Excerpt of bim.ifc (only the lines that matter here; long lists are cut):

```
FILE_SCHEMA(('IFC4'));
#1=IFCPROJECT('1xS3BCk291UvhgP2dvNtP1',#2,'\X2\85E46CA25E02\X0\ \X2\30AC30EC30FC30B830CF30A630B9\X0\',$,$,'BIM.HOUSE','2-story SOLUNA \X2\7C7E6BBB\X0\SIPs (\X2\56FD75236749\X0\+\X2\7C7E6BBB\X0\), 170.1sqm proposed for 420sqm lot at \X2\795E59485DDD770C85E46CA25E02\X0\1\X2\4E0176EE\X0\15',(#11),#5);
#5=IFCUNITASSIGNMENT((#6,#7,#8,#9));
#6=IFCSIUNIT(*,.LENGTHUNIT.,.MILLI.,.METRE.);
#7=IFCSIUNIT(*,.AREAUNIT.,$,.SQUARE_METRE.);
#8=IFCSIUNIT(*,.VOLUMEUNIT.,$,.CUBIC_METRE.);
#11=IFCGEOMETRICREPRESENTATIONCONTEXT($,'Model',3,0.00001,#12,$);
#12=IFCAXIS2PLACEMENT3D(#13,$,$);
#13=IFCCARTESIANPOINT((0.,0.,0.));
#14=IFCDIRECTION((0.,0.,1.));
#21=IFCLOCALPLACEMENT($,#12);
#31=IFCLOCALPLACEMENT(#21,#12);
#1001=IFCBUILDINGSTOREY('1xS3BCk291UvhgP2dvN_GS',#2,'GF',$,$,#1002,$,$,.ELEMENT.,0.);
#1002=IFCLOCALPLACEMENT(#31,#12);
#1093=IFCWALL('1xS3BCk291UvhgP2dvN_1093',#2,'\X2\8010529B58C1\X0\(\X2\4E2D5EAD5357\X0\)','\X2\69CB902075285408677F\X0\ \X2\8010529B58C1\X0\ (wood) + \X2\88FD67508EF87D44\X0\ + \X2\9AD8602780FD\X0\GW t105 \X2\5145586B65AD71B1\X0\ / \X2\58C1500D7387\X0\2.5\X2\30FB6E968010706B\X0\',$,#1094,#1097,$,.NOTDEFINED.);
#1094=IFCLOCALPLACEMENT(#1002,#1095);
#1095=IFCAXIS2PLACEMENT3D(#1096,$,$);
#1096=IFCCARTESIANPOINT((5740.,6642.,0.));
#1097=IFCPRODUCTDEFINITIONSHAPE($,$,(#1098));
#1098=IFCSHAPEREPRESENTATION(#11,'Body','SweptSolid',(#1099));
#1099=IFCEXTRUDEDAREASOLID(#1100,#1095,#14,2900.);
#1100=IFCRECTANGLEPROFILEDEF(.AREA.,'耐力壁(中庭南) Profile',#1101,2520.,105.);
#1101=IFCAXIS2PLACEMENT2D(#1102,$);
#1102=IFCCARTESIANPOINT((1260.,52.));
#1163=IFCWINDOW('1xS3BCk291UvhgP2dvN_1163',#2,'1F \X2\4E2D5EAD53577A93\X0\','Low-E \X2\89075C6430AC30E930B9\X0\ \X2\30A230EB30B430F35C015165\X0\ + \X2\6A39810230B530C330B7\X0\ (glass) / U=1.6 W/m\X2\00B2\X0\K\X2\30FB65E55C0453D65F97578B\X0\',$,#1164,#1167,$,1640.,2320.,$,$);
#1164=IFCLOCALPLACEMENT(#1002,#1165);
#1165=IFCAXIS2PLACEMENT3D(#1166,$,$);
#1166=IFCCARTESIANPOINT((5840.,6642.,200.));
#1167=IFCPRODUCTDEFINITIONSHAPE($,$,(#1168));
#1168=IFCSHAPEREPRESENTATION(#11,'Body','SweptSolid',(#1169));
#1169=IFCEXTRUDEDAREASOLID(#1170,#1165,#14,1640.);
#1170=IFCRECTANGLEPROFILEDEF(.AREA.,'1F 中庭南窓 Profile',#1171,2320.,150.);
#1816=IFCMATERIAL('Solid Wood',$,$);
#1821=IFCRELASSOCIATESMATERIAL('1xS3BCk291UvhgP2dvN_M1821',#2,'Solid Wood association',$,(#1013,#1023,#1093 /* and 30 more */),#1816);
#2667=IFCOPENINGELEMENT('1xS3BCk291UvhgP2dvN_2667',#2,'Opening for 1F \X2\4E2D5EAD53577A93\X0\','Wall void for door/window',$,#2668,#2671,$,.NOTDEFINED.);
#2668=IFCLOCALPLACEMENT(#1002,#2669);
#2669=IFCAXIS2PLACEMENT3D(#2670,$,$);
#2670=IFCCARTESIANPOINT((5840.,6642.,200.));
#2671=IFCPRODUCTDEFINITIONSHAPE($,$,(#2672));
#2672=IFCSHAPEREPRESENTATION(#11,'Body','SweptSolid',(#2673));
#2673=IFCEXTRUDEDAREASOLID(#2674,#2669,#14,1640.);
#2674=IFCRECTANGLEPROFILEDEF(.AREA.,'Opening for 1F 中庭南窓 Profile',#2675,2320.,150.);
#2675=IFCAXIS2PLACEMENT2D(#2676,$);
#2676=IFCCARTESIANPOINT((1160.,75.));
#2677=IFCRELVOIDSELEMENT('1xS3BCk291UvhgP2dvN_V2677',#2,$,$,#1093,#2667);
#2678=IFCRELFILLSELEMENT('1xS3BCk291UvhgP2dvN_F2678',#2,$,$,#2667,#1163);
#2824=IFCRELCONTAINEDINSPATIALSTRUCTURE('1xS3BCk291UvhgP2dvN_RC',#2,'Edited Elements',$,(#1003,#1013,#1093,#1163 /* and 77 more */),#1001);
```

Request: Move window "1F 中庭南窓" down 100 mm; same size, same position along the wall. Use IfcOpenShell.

```python
import numpy as np
import ifcopenshell
import ifcopenshell.api.geometry
import ifcopenshell.util.placement
import ifcopenshell.util.unit

model = ifcopenshell.open("bim.ifc")
unit_scale = ifcopenshell.util.unit.calculate_unit_scale(model)

window = model.by_guid("1xS3BCk291UvhgP2dvN_1163")
opening = window.FillsVoids[0].RelatingOpeningElement
dz = -100.0

shift = np.array([0.0, 0.0, dz])
# The window is not placed relative to its opening, so move both.
for product in (opening, window):
    matrix = ifcopenshell.util.placement.get_local_placement(product.ObjectPlacement)
    matrix[:3, 3] += shift
    ifcopenshell.api.geometry.edit_object_placement(model, product=product, matrix=matrix, is_si=False)

print(f"moved by {dz * unit_scale:+.3f} m")

model.write("bim_updated.ifc")
```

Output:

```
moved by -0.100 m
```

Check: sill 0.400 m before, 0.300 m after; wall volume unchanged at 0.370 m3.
